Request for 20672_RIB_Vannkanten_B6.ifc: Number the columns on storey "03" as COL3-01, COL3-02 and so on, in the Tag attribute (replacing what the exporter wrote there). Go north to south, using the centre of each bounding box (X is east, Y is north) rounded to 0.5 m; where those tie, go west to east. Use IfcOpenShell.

First a look at what the model holds.

```python
import ifcopenshell
import ifcopenshell.util.element
import ifcopenshell.util.placement

model = ifcopenshell.open("20672_RIB_Vannkanten_B6.ifc")
print(model.schema)
storey = next(s for s in model.by_type("IfcBuildingStorey") if s.Name == "03")
columns = [e for e in ifcopenshell.util.element.get_decomposition(storey) if e.is_a("IfcColumn")]
for e in sorted(columns, key=lambda e: e.id()):
    origin = ifcopenshell.util.placement.get_local_placement(e.ObjectPlacement)[:3, 3]
    print(e.id(), e.Tag, e.Name, origin.round(2) + 0.0, sep=" | ")
```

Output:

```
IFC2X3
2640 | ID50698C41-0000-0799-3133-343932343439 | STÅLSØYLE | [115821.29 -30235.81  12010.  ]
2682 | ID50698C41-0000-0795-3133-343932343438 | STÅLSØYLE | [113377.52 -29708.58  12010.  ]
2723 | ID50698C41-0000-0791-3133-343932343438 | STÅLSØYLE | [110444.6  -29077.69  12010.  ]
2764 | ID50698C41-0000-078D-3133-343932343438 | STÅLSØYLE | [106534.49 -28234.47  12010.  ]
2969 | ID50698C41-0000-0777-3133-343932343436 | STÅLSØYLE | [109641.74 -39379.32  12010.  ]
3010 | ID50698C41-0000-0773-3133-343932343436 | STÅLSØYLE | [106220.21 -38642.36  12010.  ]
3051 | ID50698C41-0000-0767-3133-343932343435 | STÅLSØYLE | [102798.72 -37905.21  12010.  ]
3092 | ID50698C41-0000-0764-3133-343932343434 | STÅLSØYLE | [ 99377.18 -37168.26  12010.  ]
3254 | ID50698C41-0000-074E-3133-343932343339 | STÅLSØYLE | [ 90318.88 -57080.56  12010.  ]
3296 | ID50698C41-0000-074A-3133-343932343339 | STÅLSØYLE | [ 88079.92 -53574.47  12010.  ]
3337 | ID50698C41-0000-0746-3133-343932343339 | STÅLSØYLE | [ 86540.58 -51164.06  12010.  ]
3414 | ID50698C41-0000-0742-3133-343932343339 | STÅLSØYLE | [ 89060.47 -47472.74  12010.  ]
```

```python
import ifcopenshell
import ifcopenshell.geom
import ifcopenshell.util.element
import ifcopenshell.util.shape

model = ifcopenshell.open("20672_RIB_Vannkanten_B6.ifc")
settings = ifcopenshell.geom.settings()
settings.set("use-world-coords", True)


def centre(element):
    shape = ifcopenshell.geom.create_shape(settings, element)
    return ifcopenshell.util.shape.get_bbox_centroid(shape.geometry)


storey = next(s for s in model.by_type("IfcBuildingStorey") if s.Name == "03")
columns = [e for e in ifcopenshell.util.element.get_decomposition(storey) if e.is_a("IfcColumn")]

# Insertion points can sit at a corner or the storey origin, so sort by the geometry (in metres).
centres = {e: centre(e) for e in columns}
columns.sort(key=lambda e: (-round(centres[e][1] / 0.5), centres[e][0]))

for i, e in enumerate(columns, start=1):
    number = f"COL3-{i:02d}"
    e.Tag = number
    print(e.id(), number)

model.write("20672_RIB_Vannkanten_B6_updated.ifc")
```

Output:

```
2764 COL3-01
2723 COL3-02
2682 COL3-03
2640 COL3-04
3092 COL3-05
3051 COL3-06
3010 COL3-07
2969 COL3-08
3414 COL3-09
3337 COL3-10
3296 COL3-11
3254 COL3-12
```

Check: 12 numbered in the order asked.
